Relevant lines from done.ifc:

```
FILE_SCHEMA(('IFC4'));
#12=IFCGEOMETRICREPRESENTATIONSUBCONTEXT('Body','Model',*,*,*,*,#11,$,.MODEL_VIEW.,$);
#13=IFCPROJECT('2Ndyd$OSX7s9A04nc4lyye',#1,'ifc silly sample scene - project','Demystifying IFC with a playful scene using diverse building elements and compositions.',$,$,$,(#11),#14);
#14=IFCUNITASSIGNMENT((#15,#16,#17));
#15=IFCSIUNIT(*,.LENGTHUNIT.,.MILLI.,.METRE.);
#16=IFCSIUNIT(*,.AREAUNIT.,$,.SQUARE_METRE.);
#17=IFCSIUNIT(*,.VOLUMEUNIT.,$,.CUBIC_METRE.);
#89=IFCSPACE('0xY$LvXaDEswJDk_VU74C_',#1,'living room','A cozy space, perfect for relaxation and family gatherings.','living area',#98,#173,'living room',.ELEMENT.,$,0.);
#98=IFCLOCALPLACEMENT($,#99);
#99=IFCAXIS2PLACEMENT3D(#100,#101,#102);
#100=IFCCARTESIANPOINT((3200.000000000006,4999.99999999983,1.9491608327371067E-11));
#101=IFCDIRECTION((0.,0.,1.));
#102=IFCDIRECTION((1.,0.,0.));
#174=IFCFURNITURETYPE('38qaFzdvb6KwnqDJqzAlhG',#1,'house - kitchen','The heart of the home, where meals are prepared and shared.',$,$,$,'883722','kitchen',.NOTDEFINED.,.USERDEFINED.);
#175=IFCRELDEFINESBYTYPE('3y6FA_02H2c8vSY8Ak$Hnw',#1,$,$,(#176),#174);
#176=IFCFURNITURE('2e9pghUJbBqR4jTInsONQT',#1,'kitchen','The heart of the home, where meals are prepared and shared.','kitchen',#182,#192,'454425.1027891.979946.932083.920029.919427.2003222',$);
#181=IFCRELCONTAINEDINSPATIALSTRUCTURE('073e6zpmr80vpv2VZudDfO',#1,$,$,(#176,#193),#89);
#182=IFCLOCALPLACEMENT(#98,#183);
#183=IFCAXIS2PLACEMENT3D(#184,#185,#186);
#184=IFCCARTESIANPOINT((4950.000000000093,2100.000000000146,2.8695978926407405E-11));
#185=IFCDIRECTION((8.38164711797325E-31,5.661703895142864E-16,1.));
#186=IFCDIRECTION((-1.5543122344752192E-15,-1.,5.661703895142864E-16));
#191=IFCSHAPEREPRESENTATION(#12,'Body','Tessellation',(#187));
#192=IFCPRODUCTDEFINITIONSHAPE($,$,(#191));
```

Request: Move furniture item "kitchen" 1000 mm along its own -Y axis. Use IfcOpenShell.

```python
import ifcopenshell
import ifcopenshell.api.geometry
import ifcopenshell.util.placement

model = ifcopenshell.open("done.ifc")

item = model.by_guid("2e9pghUJbBqR4jTInsONQT")
matrix = ifcopenshell.util.placement.get_local_placement(item.ObjectPlacement)
matrix[:3, 3] -= matrix[:3, 1] * 1000.0
ifcopenshell.api.geometry.edit_object_placement(model, product=item, matrix=matrix, is_si=False)

print(ifcopenshell.util.placement.get_local_placement(item.ObjectPlacement).round(3) + 0.0)

model.write("done_edited.ifc")
```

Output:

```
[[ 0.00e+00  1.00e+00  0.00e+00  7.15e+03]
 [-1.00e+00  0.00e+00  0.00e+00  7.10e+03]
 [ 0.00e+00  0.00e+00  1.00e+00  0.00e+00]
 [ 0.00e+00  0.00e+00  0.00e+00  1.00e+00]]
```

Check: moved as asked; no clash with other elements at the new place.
